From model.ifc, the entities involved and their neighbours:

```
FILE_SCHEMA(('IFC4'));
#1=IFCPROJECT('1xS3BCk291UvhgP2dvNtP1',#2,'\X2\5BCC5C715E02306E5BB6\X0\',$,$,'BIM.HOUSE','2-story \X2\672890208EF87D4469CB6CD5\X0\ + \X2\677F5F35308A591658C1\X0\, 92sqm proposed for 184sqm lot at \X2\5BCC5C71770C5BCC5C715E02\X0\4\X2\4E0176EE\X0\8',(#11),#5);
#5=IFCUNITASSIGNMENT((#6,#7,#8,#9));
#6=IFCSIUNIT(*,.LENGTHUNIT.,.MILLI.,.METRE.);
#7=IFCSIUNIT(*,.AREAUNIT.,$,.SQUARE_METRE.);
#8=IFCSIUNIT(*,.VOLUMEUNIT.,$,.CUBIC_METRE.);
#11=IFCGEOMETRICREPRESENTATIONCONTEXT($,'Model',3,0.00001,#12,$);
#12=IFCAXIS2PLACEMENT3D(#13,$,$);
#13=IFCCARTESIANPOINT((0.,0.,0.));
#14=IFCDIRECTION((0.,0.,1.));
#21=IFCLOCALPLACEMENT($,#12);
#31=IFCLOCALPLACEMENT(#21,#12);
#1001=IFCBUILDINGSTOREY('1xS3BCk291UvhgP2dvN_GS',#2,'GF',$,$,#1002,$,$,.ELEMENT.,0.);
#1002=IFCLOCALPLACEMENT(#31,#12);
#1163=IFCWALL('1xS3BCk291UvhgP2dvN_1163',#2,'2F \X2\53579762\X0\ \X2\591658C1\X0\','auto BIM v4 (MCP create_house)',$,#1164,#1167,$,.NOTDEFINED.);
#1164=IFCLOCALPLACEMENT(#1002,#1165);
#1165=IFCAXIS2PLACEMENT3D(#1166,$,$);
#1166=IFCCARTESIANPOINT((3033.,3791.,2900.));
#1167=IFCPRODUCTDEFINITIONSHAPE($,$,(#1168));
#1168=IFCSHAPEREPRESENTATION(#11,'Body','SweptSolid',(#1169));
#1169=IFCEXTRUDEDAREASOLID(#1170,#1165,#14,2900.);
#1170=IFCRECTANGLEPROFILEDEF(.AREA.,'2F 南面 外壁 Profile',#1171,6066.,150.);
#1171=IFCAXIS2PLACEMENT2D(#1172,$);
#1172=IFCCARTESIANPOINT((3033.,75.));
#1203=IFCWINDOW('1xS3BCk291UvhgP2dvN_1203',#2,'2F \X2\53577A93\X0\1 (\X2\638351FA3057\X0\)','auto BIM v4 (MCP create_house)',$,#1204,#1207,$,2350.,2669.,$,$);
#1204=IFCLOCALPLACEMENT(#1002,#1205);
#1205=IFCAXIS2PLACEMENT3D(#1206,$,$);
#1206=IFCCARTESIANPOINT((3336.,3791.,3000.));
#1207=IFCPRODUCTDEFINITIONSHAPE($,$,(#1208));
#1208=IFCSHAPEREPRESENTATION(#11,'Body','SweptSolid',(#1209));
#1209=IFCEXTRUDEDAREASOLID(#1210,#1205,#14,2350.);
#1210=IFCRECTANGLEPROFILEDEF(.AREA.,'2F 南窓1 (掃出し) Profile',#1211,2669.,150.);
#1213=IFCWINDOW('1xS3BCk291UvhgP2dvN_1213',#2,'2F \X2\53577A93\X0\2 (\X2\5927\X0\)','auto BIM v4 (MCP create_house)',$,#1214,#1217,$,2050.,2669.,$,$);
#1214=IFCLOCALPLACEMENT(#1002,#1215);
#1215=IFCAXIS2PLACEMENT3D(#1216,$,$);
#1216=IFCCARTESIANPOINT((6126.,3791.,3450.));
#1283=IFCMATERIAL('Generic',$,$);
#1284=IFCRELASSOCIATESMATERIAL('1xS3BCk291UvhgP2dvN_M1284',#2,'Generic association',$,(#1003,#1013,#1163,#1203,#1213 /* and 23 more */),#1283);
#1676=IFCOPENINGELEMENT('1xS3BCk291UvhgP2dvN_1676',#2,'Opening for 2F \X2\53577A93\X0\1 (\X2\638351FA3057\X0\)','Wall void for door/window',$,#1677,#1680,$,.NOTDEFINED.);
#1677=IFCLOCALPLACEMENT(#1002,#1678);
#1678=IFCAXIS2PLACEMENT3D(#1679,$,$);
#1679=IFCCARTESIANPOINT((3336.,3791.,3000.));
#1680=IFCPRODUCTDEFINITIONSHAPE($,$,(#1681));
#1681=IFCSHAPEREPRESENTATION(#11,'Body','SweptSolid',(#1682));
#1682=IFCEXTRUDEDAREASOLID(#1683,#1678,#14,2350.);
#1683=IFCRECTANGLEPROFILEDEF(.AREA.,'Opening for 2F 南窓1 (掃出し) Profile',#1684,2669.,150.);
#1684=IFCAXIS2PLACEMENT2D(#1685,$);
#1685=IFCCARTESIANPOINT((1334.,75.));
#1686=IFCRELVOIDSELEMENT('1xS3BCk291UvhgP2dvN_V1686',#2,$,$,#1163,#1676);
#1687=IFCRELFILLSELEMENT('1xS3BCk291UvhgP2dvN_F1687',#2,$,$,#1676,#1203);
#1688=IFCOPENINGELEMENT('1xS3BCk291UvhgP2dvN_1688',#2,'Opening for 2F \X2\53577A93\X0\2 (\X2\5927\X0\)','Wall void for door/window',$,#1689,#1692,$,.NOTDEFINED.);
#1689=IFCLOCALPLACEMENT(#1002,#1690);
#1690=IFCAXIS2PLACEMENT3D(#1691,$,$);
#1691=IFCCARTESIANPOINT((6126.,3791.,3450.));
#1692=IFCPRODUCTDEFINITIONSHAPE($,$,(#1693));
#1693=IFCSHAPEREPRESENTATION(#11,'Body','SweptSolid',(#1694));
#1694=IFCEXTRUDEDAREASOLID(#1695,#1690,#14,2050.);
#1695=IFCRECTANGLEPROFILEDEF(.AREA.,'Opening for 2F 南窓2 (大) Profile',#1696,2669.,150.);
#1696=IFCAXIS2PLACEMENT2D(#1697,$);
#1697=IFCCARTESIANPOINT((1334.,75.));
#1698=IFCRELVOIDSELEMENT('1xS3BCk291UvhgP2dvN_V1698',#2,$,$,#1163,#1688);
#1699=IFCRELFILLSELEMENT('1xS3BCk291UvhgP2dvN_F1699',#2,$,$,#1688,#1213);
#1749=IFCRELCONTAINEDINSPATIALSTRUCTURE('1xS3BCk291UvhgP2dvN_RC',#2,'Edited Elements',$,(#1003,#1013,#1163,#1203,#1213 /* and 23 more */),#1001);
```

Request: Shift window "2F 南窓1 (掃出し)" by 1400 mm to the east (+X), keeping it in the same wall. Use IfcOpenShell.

```python
import ifcopenshell
import ifcopenshell.api.geometry
import ifcopenshell.util.placement
import ifcopenshell.util.unit

model = ifcopenshell.open("model.ifc")
unit_scale = ifcopenshell.util.unit.calculate_unit_scale(model)

window = model.by_guid("1xS3BCk291UvhgP2dvN_1203")
opening = window.FillsVoids[0].RelatingOpeningElement
wall = opening.VoidsElements[0].RelatingBuildingElement

wall_matrix = ifcopenshell.util.placement.get_local_placement(wall.ObjectPlacement)
shift = wall_matrix[:3, 0] * 1.4 / unit_scale
before = ifcopenshell.util.placement.get_local_placement(window.ObjectPlacement)[:3, 3].copy()

# The window is not placed relative to its opening, so move both.
for product in (opening, window):
    matrix = ifcopenshell.util.placement.get_local_placement(product.ObjectPlacement)
    matrix[:3, 3] += shift
    ifcopenshell.api.geometry.edit_object_placement(model, product=product, matrix=matrix, is_si=False)

after = ifcopenshell.util.placement.get_local_placement(window.ObjectPlacement)[:3, 3]
print("window moved by", (after - before).round(3) + 0.0)

model.write("model-out.ifc")
```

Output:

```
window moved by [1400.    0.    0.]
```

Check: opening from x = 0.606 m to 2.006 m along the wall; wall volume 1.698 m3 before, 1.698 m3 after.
